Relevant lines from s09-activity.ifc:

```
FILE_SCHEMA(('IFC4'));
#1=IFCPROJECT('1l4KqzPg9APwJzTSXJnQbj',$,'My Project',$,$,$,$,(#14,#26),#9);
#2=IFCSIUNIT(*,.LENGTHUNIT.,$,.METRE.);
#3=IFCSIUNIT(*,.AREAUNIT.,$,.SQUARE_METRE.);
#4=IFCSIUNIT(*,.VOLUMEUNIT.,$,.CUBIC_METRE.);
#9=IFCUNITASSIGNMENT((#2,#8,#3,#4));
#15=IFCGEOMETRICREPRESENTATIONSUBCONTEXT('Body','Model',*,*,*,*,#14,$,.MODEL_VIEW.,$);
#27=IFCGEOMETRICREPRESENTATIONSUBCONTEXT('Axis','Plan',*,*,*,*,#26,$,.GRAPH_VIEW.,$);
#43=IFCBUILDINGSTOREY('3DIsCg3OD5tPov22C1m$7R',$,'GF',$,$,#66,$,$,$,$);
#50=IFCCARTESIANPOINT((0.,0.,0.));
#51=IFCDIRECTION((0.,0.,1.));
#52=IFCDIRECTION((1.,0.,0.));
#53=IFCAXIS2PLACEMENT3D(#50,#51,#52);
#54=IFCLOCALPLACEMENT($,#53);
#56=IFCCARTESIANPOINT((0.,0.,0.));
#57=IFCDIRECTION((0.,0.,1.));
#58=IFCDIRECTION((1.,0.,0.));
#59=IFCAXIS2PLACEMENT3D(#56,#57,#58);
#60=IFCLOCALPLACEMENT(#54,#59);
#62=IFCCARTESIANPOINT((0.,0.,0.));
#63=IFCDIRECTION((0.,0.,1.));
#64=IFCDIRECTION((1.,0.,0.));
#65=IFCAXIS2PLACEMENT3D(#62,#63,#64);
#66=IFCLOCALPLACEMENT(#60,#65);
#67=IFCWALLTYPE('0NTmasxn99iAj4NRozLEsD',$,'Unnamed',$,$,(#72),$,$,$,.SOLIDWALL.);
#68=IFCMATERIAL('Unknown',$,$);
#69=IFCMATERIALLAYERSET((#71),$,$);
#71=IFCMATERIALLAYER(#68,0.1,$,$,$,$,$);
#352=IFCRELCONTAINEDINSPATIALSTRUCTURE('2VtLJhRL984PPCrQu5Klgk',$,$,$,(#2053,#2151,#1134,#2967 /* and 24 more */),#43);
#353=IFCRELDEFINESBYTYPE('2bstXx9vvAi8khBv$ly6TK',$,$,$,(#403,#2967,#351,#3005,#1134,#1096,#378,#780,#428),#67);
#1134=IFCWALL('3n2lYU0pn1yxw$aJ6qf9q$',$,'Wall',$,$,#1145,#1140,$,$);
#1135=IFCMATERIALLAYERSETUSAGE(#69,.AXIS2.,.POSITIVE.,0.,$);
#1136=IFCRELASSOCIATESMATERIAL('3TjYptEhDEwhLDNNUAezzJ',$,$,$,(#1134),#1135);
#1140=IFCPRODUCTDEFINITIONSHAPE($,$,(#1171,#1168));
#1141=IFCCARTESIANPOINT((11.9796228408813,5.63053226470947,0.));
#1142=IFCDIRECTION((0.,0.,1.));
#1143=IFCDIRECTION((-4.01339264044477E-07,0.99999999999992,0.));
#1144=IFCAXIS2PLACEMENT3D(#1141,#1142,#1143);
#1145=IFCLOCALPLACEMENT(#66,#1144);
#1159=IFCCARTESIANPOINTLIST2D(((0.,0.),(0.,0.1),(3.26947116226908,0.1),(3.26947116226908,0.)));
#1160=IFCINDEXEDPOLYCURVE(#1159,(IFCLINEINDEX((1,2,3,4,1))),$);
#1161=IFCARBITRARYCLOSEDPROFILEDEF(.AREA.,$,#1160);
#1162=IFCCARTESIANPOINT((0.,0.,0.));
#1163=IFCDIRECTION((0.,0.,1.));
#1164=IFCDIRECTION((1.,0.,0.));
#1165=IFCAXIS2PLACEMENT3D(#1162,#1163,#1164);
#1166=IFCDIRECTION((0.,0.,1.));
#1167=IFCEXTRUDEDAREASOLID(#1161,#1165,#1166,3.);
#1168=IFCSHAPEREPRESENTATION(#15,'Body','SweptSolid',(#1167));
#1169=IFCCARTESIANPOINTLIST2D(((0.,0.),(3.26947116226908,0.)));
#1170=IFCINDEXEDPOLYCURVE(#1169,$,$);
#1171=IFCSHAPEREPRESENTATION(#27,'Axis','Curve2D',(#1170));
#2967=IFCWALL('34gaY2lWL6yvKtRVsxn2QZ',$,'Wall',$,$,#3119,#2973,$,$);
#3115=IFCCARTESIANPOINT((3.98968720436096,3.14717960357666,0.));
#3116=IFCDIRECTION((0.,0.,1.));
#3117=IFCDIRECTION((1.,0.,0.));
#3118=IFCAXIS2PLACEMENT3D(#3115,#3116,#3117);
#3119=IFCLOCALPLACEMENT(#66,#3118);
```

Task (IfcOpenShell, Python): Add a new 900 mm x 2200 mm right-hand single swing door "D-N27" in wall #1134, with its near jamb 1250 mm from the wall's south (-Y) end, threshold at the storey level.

```python
import numpy as np
import ifcopenshell
import ifcopenshell.api.feature
import ifcopenshell.api.geometry
import ifcopenshell.api.root
import ifcopenshell.api.spatial
import ifcopenshell.geom
import ifcopenshell.util.element
import ifcopenshell.util.placement
import ifcopenshell.util.representation
import ifcopenshell.util.shape
import ifcopenshell.util.unit

model = ifcopenshell.open("s09-activity.ifc")
unit_scale = ifcopenshell.util.unit.calculate_unit_scale(model)
settings = ifcopenshell.geom.settings()


def volume(element):
    """Net volume in cubic metres, openings subtracted."""
    shape = ifcopenshell.geom.create_shape(settings, element)
    return ifcopenshell.util.shape.get_volume(shape.geometry)


wall = model.by_guid("3n2lYU0pn1yxw$aJ6qf9q$")
storey = ifcopenshell.util.element.get_container(wall, ifc_class="IfcBuildingStorey")
context = ifcopenshell.util.representation.get_context(model, "Model", "Body", "MODEL_VIEW")
before = volume(wall)

width, height, from_end, sill = 0.9, 2.2, 1.25, 0.0  # metres

# The wall runs along its own X axis, and the end named is its -X end.
wall_shape = ifcopenshell.geom.create_shape(settings, wall)
x, y, z = ifcopenshell.util.shape.get_vertices(wall_shape.geometry).T
start = x.min() + from_end
face, thickness = float(y.min()), float(y.max() - y.min())
wall_matrix = ifcopenshell.util.placement.get_local_placement(wall.ObjectPlacement)
level = ifcopenshell.util.placement.get_local_placement(storey.ObjectPlacement)[2, 3]


def in_wall(x, y):
    """Placement at x, y metres in the wall's axes, at sill height."""
    matrix = wall_matrix.copy()
    matrix[:, 3] = wall_matrix @ np.array([x / unit_scale, y / unit_scale, 0.0, 1.0])
    matrix[2, 3] = level + sill / unit_scale
    return matrix


# Opening: a box that overshoots both wall faces by 50 mm.
opening = ifcopenshell.api.root.create_entity(model, ifc_class="IfcOpeningElement", predefined_type="OPENING")
box = ifcopenshell.api.geometry.add_wall_representation(
    model, context=context, length=width, height=height, thickness=thickness + 0.1
)
ifcopenshell.api.geometry.assign_representation(model, product=opening, representation=box)
ifcopenshell.api.geometry.edit_object_placement(model, product=opening, matrix=in_wall(start, face - 0.05), is_si=False)
ifcopenshell.api.feature.add_feature(model, feature=opening, element=wall)

door = ifcopenshell.api.root.create_entity(model, ifc_class="IfcDoor", name="D-N27", predefined_type="DOOR")
door.OverallWidth, door.OverallHeight = width / unit_scale, height / unit_scale
door.OperationType = "SINGLE_SWING_RIGHT"
body = ifcopenshell.api.geometry.add_door_representation(
    model,
    context=context,
    overall_width=door.OverallWidth,
    overall_height=door.OverallHeight,
    operation_type="SINGLE_SWING_RIGHT",
    lining_properties={"LiningDepth": thickness / unit_scale, "ThresholdDepth": thickness / unit_scale},
)
ifcopenshell.api.geometry.assign_representation(model, product=door, representation=body)
ifcopenshell.api.spatial.assign_container(model, products=[door], relating_structure=storey)
ifcopenshell.api.feature.add_filling(model, opening=opening, element=door)

# The lining spans the wall, so the door starts at the wall face.
ifcopenshell.api.geometry.edit_object_placement(model, product=door, matrix=in_wall(start, face), is_si=False)

after = volume(wall)

print(f"wall volume {before:.3f} -> {after:.3f} m3")

model.write("s09-activity_rev.ifc")
```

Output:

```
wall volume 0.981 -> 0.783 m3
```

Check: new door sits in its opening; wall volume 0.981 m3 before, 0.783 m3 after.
